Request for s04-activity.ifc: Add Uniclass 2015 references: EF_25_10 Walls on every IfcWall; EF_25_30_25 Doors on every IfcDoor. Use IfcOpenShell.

First a look at what the model holds.

```python
import ifcopenshell

model = ifcopenshell.open("s04-activity.ifc")
print(model.schema)
print("classifications:", [c.Name for c in model.by_type("IfcClassification")])
for ifc_class in ("IfcDoor", "IfcRoof", "IfcStair", "IfcWall", "IfcWindow"):
    print(ifc_class, len(model.by_type(ifc_class)))
```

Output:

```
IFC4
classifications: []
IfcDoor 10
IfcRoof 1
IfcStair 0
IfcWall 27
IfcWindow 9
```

```python
import ifcopenshell
import ifcopenshell.api.classification

model = ifcopenshell.open("s04-activity.ifc")

system = ifcopenshell.api.classification.add_classification(model, classification="Uniclass 2015")

codes = {
    "IfcWall": ("EF_25_10", "Walls"),
    "IfcDoor": ("EF_25_30_25", "Doors"),
}
for ifc_class, (code, name) in codes.items():
    products = model.by_type(ifc_class)
    ifcopenshell.api.classification.add_reference(
        model, products=products, classification=system, identification=code, name=name
    )
    print(code, len(products))

model.write("s04-activity_v2.ifc")
```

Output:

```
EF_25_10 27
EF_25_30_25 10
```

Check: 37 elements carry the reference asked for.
